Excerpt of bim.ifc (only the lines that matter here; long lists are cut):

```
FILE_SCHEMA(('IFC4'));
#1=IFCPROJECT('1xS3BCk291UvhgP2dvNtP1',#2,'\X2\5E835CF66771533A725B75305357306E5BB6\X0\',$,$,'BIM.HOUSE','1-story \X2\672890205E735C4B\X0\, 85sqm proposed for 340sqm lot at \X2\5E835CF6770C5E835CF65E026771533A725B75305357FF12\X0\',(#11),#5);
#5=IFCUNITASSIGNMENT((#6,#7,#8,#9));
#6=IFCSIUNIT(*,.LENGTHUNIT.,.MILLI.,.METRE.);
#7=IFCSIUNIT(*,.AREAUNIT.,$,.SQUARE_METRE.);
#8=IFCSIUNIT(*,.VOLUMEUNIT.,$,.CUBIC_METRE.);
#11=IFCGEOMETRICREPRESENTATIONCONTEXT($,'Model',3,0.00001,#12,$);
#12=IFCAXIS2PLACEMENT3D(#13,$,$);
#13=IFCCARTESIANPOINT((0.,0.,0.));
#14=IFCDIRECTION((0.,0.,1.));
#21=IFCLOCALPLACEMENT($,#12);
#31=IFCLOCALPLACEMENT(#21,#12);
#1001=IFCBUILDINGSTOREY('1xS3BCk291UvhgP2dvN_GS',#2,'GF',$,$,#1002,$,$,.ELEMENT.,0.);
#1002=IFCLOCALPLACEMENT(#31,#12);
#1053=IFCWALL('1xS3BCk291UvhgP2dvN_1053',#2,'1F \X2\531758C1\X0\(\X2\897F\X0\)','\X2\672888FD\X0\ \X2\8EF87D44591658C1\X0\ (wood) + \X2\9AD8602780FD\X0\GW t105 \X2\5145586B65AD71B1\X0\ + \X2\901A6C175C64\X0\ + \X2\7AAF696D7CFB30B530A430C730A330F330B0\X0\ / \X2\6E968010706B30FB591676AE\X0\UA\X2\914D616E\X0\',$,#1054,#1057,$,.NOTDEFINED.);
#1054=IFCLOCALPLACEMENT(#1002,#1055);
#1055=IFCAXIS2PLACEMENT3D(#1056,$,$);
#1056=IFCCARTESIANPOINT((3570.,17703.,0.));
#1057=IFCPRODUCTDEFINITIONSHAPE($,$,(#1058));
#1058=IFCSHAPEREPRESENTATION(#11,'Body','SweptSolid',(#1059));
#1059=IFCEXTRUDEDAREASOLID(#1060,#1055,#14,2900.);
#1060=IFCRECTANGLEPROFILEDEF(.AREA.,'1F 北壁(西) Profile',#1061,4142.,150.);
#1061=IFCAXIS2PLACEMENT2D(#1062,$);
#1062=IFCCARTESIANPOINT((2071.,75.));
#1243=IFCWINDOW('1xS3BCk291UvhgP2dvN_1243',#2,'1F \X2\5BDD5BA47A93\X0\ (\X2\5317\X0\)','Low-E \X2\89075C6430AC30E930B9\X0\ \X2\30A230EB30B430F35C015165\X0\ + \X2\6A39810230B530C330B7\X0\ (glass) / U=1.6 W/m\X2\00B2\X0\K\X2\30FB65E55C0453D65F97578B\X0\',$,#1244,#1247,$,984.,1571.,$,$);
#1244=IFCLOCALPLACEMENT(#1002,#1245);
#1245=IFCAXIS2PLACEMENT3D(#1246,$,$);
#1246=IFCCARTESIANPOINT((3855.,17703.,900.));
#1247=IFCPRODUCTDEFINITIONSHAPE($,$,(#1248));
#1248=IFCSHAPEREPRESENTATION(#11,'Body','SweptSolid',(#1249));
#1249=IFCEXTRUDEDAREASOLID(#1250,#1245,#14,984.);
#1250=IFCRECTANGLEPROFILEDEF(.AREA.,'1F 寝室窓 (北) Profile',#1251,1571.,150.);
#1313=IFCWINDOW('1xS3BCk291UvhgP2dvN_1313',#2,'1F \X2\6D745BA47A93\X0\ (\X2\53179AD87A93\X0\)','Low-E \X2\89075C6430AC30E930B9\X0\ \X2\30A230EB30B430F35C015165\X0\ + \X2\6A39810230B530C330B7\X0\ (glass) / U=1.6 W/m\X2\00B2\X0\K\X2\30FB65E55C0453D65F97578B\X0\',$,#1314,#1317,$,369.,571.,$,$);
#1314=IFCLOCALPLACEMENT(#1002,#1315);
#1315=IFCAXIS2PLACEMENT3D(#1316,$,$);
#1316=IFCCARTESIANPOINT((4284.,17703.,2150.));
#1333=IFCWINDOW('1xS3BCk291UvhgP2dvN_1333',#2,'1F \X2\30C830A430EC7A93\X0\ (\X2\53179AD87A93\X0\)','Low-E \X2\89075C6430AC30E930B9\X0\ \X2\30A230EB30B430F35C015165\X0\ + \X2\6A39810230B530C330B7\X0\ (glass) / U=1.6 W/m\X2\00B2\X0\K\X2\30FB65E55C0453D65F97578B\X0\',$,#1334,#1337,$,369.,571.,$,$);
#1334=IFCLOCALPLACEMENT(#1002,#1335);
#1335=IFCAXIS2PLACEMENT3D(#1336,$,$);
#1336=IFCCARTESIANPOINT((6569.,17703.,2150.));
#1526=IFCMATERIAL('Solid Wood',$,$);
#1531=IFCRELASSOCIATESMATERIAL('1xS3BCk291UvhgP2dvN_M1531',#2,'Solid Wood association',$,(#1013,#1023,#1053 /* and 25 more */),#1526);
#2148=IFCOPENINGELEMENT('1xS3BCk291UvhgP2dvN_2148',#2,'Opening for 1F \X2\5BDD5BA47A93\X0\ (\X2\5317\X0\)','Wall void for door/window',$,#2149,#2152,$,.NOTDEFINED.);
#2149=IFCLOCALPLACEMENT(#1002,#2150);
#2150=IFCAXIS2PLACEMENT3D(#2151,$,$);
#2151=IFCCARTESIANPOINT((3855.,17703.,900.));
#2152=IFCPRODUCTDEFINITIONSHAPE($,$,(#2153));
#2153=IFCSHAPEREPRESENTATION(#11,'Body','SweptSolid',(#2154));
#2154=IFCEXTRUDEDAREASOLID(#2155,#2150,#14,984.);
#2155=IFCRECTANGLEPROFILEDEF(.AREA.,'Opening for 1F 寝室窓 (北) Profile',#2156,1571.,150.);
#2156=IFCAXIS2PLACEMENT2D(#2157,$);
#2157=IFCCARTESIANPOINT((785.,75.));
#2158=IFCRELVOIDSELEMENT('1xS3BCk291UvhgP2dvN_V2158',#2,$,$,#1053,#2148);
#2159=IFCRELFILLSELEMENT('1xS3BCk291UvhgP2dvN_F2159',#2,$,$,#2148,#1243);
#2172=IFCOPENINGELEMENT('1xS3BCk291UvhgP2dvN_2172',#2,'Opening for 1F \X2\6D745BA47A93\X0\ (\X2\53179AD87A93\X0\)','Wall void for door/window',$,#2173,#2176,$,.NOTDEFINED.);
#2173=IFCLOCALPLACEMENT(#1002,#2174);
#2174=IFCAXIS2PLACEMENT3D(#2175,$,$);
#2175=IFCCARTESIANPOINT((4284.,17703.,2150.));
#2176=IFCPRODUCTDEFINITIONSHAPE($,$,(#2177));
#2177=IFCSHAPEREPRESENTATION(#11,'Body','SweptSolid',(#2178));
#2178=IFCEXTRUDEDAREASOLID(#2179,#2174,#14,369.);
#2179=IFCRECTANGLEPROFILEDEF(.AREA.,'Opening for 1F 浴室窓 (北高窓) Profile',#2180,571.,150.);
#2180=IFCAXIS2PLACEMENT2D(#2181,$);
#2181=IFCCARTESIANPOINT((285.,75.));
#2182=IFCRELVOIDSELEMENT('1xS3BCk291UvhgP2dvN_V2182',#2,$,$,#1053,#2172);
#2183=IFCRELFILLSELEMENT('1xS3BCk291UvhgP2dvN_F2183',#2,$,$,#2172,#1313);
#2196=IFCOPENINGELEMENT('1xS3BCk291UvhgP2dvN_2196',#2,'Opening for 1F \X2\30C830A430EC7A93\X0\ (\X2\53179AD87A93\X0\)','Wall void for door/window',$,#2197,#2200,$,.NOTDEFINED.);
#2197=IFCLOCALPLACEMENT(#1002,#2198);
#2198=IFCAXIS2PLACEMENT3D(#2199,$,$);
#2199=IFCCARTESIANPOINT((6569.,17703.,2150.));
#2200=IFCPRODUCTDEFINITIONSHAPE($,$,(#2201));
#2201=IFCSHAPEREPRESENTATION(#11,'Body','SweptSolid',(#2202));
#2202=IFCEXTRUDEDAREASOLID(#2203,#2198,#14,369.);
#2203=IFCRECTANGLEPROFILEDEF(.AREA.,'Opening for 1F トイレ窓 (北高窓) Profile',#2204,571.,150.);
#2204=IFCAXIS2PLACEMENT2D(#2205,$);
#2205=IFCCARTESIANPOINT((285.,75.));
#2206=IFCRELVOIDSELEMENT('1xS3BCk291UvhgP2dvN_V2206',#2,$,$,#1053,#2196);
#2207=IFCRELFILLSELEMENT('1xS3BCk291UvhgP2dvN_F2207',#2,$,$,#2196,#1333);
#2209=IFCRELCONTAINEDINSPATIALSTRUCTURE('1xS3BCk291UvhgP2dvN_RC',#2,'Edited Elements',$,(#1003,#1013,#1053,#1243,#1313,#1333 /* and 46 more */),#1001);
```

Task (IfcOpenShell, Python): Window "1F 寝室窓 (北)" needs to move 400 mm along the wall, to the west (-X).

```python
import ifcopenshell
import ifcopenshell.api.geometry
import ifcopenshell.util.placement
import ifcopenshell.util.unit

model = ifcopenshell.open("bim.ifc")
unit_scale = ifcopenshell.util.unit.calculate_unit_scale(model)

window = model.by_guid("1xS3BCk291UvhgP2dvN_1243")
opening = window.FillsVoids[0].RelatingOpeningElement
wall = opening.VoidsElements[0].RelatingBuildingElement

wall_matrix = ifcopenshell.util.placement.get_local_placement(wall.ObjectPlacement)
shift = wall_matrix[:3, 0] * -0.4 / unit_scale
before = ifcopenshell.util.placement.get_local_placement(window.ObjectPlacement)[:3, 3].copy()

# The window is not placed relative to its opening, so move both.
for product in (opening, window):
    matrix = ifcopenshell.util.placement.get_local_placement(product.ObjectPlacement)
    matrix[:3, 3] += shift
    ifcopenshell.api.geometry.edit_object_placement(model, product=product, matrix=matrix, is_si=False)

after = ifcopenshell.util.placement.get_local_placement(window.ObjectPlacement)[:3, 3]
print("window moved by", (after - before).round(3) + 0.0)

model.write("bim_updated.ifc")
```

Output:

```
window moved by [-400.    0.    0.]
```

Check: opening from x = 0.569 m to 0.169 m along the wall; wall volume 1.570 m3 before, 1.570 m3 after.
